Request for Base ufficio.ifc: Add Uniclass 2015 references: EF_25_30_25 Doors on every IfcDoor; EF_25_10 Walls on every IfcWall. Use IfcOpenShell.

First a look at what the model holds.

```python
import ifcopenshell

model = ifcopenshell.open("Base ufficio.ifc")
print(model.schema)
print("classifications:", [c.Name for c in model.by_type("IfcClassification")])
for ifc_class in ("IfcDoor", "IfcRoof", "IfcStair", "IfcWall", "IfcWindow"):
    print(ifc_class, len(model.by_type(ifc_class)))
```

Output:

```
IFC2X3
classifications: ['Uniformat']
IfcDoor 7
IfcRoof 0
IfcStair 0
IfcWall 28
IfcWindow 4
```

```python
import ifcopenshell
import ifcopenshell.api.classification

model = ifcopenshell.open("Base ufficio.ifc")

# IFC2X3 requires Source and Edition and has no link from the project to the system.
system = model.create_entity("IfcClassification", Source="NBS", Edition="2015", Name="Uniclass 2015")

codes = {
    "IfcDoor": ("EF_25_30_25", "Doors"),
    "IfcWall": ("EF_25_10", "Walls"),
}
for ifc_class, (code, name) in codes.items():
    products = model.by_type(ifc_class)
    ifcopenshell.api.classification.add_reference(
        model, products=products, classification=system, identification=code, name=name
    )
    print(code, len(products))

model.write("Base ufficio-out.ifc")
```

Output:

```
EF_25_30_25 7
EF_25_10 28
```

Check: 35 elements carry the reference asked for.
